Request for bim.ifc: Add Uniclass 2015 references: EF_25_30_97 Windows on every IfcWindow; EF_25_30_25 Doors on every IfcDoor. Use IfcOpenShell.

First a look at what the model holds.

```python
import ifcopenshell

model = ifcopenshell.open("bim.ifc")
print(model.schema)
print("classifications:", [c.Name for c in model.by_type("IfcClassification")])
for ifc_class in ("IfcDoor", "IfcRoof", "IfcStair", "IfcWall", "IfcWindow"):
    print(ifc_class, len(model.by_type(ifc_class)))
```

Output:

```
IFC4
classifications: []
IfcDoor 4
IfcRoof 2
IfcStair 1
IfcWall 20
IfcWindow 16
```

```python
import ifcopenshell
import ifcopenshell.api.classification

model = ifcopenshell.open("bim.ifc")

system = ifcopenshell.api.classification.add_classification(model, classification="Uniclass 2015")

codes = {
    "IfcWindow": ("EF_25_30_97", "Windows"),
    "IfcDoor": ("EF_25_30_25", "Doors"),
}
for ifc_class, (code, name) in codes.items():
    products = model.by_type(ifc_class)
    ifcopenshell.api.classification.add_reference(
        model, products=products, classification=system, identification=code, name=name
    )
    print(code, len(products))

model.write("bim_v2.ifc")
```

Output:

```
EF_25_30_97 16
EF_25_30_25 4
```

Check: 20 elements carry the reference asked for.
